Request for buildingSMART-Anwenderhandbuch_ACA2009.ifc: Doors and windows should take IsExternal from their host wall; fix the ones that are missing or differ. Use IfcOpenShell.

First a look at what the model holds.

```python
import ifcopenshell
import ifcopenshell.util.element

model = ifcopenshell.open("buildingSMART-Anwenderhandbuch_ACA2009.ifc")
print(model.schema)
seen = {}
for e in model.by_type("IfcDoor") + model.by_type("IfcWindow"):
    if not e.FillsVoids:
        continue
    host = e.FillsVoids[0].RelatingOpeningElement.VoidsElements[0].RelatingBuildingElement
    own = ifcopenshell.util.element.get_pset(e, f"Pset_{e.is_a()[3:].removesuffix('StandardCase')}Common", "IsExternal")
    wall = ifcopenshell.util.element.get_pset(host, "Pset_WallCommon", "IsExternal")
    seen[e.is_a(), own, wall] = seen.get((e.is_a(), own, wall), 0) + 1
for (cls, own, wall), count in sorted(seen.items(), key=str):
    print(count, cls, "IsExternal:", own, "| host wall:", wall)
```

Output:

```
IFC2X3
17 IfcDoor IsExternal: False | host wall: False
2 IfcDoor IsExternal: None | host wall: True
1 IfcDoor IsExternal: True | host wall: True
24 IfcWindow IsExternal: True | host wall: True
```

```python
import ifcopenshell
import ifcopenshell.api.pset
import ifcopenshell.util.element

model = ifcopenshell.open("buildingSMART-Anwenderhandbuch_ACA2009.ifc")

count = 0
for ifc_class, pset_name in (("IfcDoor", "Pset_DoorCommon"), ("IfcWindow", "Pset_WindowCommon")):
    for e in model.by_type(ifc_class):
        if not e.FillsVoids:
            continue
        host = e.FillsVoids[0].RelatingOpeningElement.VoidsElements[0].RelatingBuildingElement
        external = ifcopenshell.util.element.get_pset(host, "Pset_WallCommon", "IsExternal")
        if external is None or ifcopenshell.util.element.get_pset(e, pset_name, "IsExternal") == external:
            continue
        pset = ifcopenshell.api.pset.add_pset(model, product=e, name=pset_name)
        ifcopenshell.api.pset.edit_pset(model, pset=pset, properties={"IsExternal": external})
        count += 1

print(count, "updated")

model.write("buildingSMART-Anwenderhandbuch_ACA2009_edited.ifc")
```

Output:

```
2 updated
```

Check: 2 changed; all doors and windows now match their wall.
